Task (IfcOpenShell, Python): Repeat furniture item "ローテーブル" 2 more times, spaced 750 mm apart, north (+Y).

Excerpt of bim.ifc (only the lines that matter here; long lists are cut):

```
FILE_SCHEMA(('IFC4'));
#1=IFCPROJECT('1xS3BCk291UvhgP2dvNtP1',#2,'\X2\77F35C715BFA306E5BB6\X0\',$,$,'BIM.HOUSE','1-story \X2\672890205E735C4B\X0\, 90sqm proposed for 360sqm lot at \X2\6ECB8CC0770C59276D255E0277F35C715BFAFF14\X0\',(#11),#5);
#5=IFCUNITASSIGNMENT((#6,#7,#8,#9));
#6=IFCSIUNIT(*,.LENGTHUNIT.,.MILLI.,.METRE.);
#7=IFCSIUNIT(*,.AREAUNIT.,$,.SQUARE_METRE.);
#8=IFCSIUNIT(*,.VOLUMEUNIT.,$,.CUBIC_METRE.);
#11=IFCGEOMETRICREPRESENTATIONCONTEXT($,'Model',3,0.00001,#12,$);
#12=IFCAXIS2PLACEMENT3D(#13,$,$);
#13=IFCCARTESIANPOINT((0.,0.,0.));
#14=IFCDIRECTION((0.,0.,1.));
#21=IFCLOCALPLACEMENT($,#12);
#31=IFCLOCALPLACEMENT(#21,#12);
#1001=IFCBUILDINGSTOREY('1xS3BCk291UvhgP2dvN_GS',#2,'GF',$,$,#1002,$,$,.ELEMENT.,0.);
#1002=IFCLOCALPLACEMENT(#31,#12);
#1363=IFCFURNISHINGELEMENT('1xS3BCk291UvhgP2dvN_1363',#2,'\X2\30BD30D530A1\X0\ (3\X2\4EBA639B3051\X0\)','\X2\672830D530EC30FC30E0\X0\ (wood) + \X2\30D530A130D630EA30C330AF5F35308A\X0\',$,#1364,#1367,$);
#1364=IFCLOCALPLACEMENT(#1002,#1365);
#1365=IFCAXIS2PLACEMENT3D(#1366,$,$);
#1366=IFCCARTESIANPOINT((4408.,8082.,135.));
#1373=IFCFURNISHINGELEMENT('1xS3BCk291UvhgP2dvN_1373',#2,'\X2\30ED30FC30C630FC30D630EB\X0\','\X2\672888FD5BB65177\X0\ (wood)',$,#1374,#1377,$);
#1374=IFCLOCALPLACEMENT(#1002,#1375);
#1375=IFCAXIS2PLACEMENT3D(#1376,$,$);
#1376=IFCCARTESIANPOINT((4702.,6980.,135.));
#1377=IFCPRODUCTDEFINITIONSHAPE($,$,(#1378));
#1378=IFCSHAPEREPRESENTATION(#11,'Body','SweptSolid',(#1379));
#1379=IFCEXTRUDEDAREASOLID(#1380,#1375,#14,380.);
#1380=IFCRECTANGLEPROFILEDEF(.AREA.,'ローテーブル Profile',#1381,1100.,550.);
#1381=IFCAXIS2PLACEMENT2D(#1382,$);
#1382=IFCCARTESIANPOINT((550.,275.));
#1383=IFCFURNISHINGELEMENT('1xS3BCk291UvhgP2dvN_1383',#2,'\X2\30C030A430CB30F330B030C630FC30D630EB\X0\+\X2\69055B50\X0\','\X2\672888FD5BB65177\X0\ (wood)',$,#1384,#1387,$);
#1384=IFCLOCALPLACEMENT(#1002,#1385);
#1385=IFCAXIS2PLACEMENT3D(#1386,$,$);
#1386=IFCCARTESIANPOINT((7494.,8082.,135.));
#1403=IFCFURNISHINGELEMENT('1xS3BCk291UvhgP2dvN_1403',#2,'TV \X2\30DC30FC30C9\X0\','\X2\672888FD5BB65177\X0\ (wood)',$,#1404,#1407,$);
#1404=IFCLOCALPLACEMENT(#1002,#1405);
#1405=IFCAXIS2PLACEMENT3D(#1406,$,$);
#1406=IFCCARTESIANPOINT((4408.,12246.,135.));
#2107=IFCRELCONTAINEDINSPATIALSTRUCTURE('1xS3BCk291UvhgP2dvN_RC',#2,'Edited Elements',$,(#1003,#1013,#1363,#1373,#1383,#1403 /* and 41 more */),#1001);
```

```python
import numpy as np
import ifcopenshell
import ifcopenshell.api.geometry
import ifcopenshell.api.root
import ifcopenshell.util.element
import ifcopenshell.util.placement

model = ifcopenshell.open("bim.ifc")


def reuse_history(source, copy):
    """copy_class also copies each property set's owner history, people and application; keep the originals."""
    for rel in copy.IsDefinedBy:
        if rel.is_a("IfcRelDefinesByProperties") and (history := rel.RelatingPropertyDefinition.OwnerHistory):
            rel.RelatingPropertyDefinition.OwnerHistory = source.OwnerHistory
            ifcopenshell.util.element.remove_deep2(model, history)


source = model.by_guid("1xS3BCk291UvhgP2dvN_1373")
base = ifcopenshell.util.placement.get_local_placement(source.ObjectPlacement)
step = np.array([0.0, 1.0, 0.0]) * 750.0

for i in range(1, 3):
    copy = ifcopenshell.api.root.copy_class(model, product=source)
    copy.Representation = ifcopenshell.util.element.copy_deep(
        model, source.Representation, exclude=["IfcGeometricRepresentationContext", "IfcRepresentationMap"]
    )
    reuse_history(source, copy)
    matrix = base.copy()
    matrix[:3, 3] += i * step
    print("added at", matrix[:3, 3].round(3) + 0.0)
    ifcopenshell.api.geometry.edit_object_placement(model, product=copy, matrix=matrix, is_si=False)

model.write("bim-out.ifc")
```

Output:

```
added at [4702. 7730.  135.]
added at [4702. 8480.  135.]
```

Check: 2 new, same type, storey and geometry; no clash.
